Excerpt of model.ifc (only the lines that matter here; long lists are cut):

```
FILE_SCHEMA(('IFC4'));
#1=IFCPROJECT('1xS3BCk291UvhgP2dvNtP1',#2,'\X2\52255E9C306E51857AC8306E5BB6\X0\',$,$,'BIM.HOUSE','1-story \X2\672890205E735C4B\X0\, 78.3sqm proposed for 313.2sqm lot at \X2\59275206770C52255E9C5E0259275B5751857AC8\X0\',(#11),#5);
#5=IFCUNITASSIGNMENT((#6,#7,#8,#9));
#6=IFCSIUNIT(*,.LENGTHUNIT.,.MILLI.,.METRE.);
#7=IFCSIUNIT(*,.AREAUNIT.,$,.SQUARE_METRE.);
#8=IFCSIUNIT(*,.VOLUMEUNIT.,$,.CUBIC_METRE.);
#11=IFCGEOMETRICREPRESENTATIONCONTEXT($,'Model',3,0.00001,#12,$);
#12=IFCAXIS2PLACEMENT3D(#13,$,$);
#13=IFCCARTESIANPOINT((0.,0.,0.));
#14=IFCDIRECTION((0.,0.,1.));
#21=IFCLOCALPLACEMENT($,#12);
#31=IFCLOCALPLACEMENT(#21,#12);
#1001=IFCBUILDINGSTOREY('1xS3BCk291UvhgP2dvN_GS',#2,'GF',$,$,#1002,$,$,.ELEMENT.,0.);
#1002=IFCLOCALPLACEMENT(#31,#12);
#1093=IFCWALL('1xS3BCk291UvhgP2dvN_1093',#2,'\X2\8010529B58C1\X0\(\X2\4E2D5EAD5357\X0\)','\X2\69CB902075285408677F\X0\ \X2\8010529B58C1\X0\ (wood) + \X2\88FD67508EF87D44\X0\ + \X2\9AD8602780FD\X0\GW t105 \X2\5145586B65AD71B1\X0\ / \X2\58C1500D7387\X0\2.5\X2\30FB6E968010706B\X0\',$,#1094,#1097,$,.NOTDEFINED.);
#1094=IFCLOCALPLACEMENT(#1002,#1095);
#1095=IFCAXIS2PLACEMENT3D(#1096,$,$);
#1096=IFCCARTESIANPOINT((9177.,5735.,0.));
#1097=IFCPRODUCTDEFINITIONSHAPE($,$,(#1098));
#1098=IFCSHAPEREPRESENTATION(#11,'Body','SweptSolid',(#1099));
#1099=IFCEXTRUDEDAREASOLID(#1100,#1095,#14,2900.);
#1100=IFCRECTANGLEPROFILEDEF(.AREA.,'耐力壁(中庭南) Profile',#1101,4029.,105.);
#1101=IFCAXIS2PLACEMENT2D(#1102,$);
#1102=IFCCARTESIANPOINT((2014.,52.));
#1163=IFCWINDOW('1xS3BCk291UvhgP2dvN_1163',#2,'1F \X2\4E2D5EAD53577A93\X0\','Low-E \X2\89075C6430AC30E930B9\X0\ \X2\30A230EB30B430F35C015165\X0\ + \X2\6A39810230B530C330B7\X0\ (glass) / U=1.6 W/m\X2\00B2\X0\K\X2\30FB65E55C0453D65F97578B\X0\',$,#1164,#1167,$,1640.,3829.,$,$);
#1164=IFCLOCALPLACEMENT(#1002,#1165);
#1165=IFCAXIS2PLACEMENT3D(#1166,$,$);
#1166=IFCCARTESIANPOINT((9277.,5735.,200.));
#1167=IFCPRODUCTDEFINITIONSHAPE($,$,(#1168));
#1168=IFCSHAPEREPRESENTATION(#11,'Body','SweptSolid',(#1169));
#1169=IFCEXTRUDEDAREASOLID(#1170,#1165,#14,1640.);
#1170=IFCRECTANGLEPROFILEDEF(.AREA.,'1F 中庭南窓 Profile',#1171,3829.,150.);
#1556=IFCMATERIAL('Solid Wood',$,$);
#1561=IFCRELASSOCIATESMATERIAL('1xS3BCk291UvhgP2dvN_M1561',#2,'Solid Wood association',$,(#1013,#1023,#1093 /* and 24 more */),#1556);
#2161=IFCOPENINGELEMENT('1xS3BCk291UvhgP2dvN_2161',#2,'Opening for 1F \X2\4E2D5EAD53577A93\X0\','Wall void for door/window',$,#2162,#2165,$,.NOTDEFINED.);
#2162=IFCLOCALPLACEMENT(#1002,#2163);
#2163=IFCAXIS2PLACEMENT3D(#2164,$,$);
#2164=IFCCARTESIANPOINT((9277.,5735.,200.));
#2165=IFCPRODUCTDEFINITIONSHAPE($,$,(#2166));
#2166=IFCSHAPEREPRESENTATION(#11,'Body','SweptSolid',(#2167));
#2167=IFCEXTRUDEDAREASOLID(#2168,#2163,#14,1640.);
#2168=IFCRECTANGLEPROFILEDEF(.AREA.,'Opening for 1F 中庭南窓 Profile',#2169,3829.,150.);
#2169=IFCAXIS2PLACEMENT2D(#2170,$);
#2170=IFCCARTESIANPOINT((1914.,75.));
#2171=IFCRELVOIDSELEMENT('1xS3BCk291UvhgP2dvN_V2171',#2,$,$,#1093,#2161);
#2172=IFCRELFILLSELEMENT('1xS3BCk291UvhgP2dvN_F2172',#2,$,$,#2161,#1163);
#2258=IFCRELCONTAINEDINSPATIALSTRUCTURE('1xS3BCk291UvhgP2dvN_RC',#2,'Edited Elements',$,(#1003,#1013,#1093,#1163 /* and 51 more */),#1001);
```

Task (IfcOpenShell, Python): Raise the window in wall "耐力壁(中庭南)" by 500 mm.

```python
import numpy as np
import ifcopenshell
import ifcopenshell.api.geometry
import ifcopenshell.util.placement
import ifcopenshell.util.unit

model = ifcopenshell.open("model.ifc")
unit_scale = ifcopenshell.util.unit.calculate_unit_scale(model)

window = model.by_id(1163)
opening = window.FillsVoids[0].RelatingOpeningElement
dz = 0.5 / unit_scale

shift = np.array([0.0, 0.0, dz])
# The window is not placed relative to its opening, so move both.
for product in (opening, window):
    matrix = ifcopenshell.util.placement.get_local_placement(product.ObjectPlacement)
    matrix[:3, 3] += shift
    ifcopenshell.api.geometry.edit_object_placement(model, product=product, matrix=matrix, is_si=False)

print(f"moved by {dz * unit_scale:+.3f} m")

model.write("model_v2.ifc")
```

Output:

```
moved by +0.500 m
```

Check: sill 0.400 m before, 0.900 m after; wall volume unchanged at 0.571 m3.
